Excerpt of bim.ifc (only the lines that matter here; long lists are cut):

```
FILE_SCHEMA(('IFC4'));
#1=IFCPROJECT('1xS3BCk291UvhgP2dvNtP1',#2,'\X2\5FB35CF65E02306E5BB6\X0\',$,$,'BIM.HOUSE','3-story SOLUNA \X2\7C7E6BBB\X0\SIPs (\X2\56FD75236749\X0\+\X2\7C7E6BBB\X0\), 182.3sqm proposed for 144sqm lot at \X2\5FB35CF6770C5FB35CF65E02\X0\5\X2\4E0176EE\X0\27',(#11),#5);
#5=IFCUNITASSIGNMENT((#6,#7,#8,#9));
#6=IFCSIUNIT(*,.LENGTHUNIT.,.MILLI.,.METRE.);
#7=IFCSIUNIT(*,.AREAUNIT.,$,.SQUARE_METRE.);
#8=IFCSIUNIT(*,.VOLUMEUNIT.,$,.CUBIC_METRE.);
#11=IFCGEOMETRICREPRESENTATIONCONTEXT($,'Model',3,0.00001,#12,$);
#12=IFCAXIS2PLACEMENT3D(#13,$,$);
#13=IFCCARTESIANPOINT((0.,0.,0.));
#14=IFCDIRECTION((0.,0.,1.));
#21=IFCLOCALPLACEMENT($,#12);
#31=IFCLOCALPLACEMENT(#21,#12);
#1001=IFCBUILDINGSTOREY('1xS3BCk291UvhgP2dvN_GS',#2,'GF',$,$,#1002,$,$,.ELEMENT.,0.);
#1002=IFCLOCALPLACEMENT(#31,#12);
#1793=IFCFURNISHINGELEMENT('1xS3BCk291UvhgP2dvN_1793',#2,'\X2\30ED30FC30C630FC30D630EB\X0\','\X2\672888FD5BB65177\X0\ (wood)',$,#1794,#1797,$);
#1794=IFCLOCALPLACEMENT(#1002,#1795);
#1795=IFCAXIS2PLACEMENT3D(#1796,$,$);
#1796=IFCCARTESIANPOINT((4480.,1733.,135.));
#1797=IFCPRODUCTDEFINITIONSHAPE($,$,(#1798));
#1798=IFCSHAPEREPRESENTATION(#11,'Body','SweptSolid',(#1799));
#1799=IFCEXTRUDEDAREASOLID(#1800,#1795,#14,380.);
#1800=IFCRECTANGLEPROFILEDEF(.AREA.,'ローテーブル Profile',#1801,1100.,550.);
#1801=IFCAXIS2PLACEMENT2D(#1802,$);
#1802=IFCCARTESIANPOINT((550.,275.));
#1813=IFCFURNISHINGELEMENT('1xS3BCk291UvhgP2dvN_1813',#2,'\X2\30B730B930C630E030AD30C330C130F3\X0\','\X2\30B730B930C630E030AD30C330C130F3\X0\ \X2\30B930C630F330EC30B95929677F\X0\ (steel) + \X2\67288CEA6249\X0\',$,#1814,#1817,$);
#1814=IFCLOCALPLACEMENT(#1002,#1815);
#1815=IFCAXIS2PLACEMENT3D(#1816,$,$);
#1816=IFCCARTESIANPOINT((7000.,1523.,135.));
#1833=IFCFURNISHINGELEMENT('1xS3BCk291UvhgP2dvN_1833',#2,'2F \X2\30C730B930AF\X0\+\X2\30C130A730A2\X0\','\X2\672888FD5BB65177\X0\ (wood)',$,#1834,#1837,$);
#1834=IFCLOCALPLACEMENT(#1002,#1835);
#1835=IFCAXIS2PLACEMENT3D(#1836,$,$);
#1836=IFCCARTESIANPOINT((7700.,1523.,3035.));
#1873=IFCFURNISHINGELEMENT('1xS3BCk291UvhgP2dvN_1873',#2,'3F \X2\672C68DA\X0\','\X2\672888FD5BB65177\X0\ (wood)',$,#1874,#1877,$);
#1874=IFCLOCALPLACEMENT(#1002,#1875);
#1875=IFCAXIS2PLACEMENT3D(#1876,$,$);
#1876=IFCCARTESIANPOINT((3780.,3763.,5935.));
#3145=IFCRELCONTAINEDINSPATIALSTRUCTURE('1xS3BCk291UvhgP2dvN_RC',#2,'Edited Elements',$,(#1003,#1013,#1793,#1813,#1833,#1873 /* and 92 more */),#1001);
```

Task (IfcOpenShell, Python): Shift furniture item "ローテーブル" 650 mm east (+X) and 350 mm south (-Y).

```python
import ifcopenshell
import ifcopenshell.api.geometry
import ifcopenshell.util.placement

model = ifcopenshell.open("bim.ifc")

item = model.by_id(1793)
matrix = ifcopenshell.util.placement.get_local_placement(item.ObjectPlacement)
matrix[0, 3] += 650.0
matrix[1, 3] -= 350.0
ifcopenshell.api.geometry.edit_object_placement(model, product=item, matrix=matrix, is_si=False)

print(ifcopenshell.util.placement.get_local_placement(item.ObjectPlacement).round(3) + 0.0)

model.write("bim-out.ifc")
```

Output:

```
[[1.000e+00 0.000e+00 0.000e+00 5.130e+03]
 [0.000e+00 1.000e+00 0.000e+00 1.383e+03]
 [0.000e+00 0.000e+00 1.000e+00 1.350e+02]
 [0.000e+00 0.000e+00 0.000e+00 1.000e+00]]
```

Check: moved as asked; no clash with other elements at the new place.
